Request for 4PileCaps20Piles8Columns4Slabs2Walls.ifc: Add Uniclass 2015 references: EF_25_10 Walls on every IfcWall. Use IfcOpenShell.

First a look at what the model holds.

```python
import ifcopenshell

model = ifcopenshell.open("4PileCaps20Piles8Columns4Slabs2Walls.ifc")
print(model.schema)
print("classifications:", [c.Name for c in model.by_type("IfcClassification")])
for ifc_class in ("IfcDoor", "IfcRoof", "IfcStair", "IfcWall", "IfcWindow"):
    print(ifc_class, len(model.by_type(ifc_class)))
```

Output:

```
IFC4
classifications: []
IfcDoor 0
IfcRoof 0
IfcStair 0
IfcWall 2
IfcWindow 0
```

```python
import ifcopenshell
import ifcopenshell.api.classification

model = ifcopenshell.open("4PileCaps20Piles8Columns4Slabs2Walls.ifc")

system = ifcopenshell.api.classification.add_classification(model, classification="Uniclass 2015")

codes = {
    "IfcWall": ("EF_25_10", "Walls"),
}
for ifc_class, (code, name) in codes.items():
    products = model.by_type(ifc_class)
    ifcopenshell.api.classification.add_reference(
        model, products=products, classification=system, identification=code, name=name
    )
    print(code, len(products))

model.write("4PileCaps20Piles8Columns4Slabs2Walls_edited.ifc")
```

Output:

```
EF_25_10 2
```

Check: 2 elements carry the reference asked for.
